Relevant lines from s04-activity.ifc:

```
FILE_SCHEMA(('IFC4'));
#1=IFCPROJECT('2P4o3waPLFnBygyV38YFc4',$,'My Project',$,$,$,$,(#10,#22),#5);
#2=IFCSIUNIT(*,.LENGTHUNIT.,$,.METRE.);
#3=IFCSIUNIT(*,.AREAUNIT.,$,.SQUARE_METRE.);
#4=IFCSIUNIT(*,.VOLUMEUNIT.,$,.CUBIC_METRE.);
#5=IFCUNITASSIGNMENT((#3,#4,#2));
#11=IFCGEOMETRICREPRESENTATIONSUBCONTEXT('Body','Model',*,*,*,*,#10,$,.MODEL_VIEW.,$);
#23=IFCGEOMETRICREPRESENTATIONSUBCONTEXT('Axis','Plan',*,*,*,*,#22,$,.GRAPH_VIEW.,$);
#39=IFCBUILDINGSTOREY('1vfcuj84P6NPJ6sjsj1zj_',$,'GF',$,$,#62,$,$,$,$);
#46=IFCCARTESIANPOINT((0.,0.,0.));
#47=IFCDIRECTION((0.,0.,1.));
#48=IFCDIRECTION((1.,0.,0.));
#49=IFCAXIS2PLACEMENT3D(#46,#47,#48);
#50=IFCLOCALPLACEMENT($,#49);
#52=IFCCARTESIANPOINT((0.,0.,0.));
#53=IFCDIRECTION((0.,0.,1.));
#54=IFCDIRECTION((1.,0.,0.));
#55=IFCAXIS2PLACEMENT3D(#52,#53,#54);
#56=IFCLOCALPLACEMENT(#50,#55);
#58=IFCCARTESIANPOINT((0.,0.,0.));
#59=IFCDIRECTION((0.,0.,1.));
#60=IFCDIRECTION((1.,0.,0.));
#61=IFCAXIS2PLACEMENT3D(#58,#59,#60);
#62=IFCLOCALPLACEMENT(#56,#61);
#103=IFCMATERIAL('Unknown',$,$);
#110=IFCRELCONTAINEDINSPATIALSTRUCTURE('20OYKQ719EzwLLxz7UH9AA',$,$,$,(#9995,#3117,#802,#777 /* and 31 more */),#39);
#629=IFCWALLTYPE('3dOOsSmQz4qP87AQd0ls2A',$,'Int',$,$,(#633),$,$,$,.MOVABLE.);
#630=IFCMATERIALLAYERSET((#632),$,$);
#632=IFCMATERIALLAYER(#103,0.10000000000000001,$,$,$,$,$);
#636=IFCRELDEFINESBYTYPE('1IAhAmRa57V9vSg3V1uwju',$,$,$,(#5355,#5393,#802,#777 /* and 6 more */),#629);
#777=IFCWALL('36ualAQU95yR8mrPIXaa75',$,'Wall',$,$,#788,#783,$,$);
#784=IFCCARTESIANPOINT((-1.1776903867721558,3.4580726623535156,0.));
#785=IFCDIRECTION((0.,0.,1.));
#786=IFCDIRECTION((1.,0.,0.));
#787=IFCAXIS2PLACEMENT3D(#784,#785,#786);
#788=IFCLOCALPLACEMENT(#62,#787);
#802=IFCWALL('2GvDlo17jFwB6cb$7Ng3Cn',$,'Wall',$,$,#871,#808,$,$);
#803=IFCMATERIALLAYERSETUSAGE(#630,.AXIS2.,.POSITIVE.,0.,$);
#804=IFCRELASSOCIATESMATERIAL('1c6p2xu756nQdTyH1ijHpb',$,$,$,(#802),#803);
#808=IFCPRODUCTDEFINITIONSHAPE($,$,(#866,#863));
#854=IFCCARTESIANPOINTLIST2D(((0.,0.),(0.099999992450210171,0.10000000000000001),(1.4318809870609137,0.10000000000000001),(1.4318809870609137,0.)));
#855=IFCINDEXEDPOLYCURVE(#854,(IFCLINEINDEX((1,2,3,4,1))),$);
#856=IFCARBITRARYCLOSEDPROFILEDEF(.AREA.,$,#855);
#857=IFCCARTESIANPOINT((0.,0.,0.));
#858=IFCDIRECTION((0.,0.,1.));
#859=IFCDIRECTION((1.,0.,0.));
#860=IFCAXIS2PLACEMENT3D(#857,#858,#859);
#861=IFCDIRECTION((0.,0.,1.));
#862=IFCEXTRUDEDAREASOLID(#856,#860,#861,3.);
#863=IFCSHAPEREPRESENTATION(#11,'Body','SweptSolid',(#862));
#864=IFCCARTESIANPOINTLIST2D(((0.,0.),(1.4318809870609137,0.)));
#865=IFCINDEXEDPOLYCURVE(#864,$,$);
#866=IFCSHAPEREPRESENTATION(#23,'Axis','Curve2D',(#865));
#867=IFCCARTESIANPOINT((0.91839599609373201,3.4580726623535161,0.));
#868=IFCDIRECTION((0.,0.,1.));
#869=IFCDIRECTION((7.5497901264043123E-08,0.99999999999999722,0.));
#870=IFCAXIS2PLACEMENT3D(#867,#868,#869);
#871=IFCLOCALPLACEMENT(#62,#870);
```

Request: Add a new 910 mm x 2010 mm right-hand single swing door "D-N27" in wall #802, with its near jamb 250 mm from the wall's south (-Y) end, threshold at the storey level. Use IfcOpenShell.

```python
import numpy as np
import ifcopenshell
import ifcopenshell.api.feature
import ifcopenshell.api.geometry
import ifcopenshell.api.root
import ifcopenshell.api.spatial
import ifcopenshell.geom
import ifcopenshell.util.element
import ifcopenshell.util.placement
import ifcopenshell.util.representation
import ifcopenshell.util.shape
import ifcopenshell.util.unit

model = ifcopenshell.open("s04-activity.ifc")
unit_scale = ifcopenshell.util.unit.calculate_unit_scale(model)
settings = ifcopenshell.geom.settings()


def volume(element):
    """Net volume in cubic metres, openings subtracted."""
    shape = ifcopenshell.geom.create_shape(settings, element)
    return ifcopenshell.util.shape.get_volume(shape.geometry)


wall = model.by_id(802)
storey = ifcopenshell.util.element.get_container(wall, ifc_class="IfcBuildingStorey")
context = ifcopenshell.util.representation.get_context(model, "Model", "Body", "MODEL_VIEW")
before = volume(wall)

width, height, from_end, sill = 0.91, 2.01, 0.25, 0.0  # metres

# The wall runs along its own X axis, and the end named is its -X end.
wall_shape = ifcopenshell.geom.create_shape(settings, wall)
x, y, z = ifcopenshell.util.shape.get_vertices(wall_shape.geometry).T
start = x.min() + from_end
face, thickness = float(y.min()), float(y.max() - y.min())
wall_matrix = ifcopenshell.util.placement.get_local_placement(wall.ObjectPlacement)
level = ifcopenshell.util.placement.get_local_placement(storey.ObjectPlacement)[2, 3]


def in_wall(x, y):
    """Placement at x, y metres in the wall's axes, at sill height."""
    matrix = wall_matrix.copy()
    matrix[:, 3] = wall_matrix @ np.array([x / unit_scale, y / unit_scale, 0.0, 1.0])
    matrix[2, 3] = level + sill / unit_scale
    return matrix


# Opening: a box that overshoots both wall faces by 50 mm.
opening = ifcopenshell.api.root.create_entity(model, ifc_class="IfcOpeningElement", predefined_type="OPENING")
box = ifcopenshell.api.geometry.add_wall_representation(
    model, context=context, length=width, height=height, thickness=thickness + 0.1
)
ifcopenshell.api.geometry.assign_representation(model, product=opening, representation=box)
ifcopenshell.api.geometry.edit_object_placement(model, product=opening, matrix=in_wall(start, face - 0.05), is_si=False)
ifcopenshell.api.feature.add_feature(model, feature=opening, element=wall)

door = ifcopenshell.api.root.create_entity(model, ifc_class="IfcDoor", name="D-N27", predefined_type="DOOR")
door.OverallWidth, door.OverallHeight = width / unit_scale, height / unit_scale
door.OperationType = "SINGLE_SWING_RIGHT"
body = ifcopenshell.api.geometry.add_door_representation(
    model,
    context=context,
    overall_width=door.OverallWidth,
    overall_height=door.OverallHeight,
    operation_type="SINGLE_SWING_RIGHT",
    lining_properties={"LiningDepth": thickness / unit_scale, "ThresholdDepth": thickness / unit_scale},
)
ifcopenshell.api.geometry.assign_representation(model, product=door, representation=body)
ifcopenshell.api.spatial.assign_container(model, products=[door], relating_structure=storey)
ifcopenshell.api.feature.add_filling(model, opening=opening, element=door)

# The lining spans the wall, so the door starts at the wall face.
ifcopenshell.api.geometry.edit_object_placement(model, product=door, matrix=in_wall(start, face), is_si=False)

after = volume(wall)

print(f"wall volume {before:.3f} -> {after:.3f} m3")

model.write("s04-activity_updated.ifc")
```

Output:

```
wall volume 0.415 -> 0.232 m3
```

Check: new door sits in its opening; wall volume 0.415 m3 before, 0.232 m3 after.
